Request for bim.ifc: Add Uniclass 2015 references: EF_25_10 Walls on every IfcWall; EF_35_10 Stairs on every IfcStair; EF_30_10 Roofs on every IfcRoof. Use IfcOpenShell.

First a look at what the model holds.

```python
import ifcopenshell

model = ifcopenshell.open("bim.ifc")
print(model.schema)
print("classifications:", [c.Name for c in model.by_type("IfcClassification")])
for ifc_class in ("IfcDoor", "IfcRoof", "IfcStair", "IfcWall", "IfcWindow"):
    print(ifc_class, len(model.by_type(ifc_class)))
```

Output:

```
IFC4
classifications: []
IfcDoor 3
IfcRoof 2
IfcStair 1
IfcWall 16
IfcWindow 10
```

```python
import ifcopenshell
import ifcopenshell.api.classification

model = ifcopenshell.open("bim.ifc")

system = ifcopenshell.api.classification.add_classification(model, classification="Uniclass 2015")

codes = {
    "IfcWall": ("EF_25_10", "Walls"),
    "IfcStair": ("EF_35_10", "Stairs"),
    "IfcRoof": ("EF_30_10", "Roofs"),
}
for ifc_class, (code, name) in codes.items():
    products = model.by_type(ifc_class)
    ifcopenshell.api.classification.add_reference(
        model, products=products, classification=system, identification=code, name=name
    )
    print(code, len(products))

model.write("bim_updated.ifc")
```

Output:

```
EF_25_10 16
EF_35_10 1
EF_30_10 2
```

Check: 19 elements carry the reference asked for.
